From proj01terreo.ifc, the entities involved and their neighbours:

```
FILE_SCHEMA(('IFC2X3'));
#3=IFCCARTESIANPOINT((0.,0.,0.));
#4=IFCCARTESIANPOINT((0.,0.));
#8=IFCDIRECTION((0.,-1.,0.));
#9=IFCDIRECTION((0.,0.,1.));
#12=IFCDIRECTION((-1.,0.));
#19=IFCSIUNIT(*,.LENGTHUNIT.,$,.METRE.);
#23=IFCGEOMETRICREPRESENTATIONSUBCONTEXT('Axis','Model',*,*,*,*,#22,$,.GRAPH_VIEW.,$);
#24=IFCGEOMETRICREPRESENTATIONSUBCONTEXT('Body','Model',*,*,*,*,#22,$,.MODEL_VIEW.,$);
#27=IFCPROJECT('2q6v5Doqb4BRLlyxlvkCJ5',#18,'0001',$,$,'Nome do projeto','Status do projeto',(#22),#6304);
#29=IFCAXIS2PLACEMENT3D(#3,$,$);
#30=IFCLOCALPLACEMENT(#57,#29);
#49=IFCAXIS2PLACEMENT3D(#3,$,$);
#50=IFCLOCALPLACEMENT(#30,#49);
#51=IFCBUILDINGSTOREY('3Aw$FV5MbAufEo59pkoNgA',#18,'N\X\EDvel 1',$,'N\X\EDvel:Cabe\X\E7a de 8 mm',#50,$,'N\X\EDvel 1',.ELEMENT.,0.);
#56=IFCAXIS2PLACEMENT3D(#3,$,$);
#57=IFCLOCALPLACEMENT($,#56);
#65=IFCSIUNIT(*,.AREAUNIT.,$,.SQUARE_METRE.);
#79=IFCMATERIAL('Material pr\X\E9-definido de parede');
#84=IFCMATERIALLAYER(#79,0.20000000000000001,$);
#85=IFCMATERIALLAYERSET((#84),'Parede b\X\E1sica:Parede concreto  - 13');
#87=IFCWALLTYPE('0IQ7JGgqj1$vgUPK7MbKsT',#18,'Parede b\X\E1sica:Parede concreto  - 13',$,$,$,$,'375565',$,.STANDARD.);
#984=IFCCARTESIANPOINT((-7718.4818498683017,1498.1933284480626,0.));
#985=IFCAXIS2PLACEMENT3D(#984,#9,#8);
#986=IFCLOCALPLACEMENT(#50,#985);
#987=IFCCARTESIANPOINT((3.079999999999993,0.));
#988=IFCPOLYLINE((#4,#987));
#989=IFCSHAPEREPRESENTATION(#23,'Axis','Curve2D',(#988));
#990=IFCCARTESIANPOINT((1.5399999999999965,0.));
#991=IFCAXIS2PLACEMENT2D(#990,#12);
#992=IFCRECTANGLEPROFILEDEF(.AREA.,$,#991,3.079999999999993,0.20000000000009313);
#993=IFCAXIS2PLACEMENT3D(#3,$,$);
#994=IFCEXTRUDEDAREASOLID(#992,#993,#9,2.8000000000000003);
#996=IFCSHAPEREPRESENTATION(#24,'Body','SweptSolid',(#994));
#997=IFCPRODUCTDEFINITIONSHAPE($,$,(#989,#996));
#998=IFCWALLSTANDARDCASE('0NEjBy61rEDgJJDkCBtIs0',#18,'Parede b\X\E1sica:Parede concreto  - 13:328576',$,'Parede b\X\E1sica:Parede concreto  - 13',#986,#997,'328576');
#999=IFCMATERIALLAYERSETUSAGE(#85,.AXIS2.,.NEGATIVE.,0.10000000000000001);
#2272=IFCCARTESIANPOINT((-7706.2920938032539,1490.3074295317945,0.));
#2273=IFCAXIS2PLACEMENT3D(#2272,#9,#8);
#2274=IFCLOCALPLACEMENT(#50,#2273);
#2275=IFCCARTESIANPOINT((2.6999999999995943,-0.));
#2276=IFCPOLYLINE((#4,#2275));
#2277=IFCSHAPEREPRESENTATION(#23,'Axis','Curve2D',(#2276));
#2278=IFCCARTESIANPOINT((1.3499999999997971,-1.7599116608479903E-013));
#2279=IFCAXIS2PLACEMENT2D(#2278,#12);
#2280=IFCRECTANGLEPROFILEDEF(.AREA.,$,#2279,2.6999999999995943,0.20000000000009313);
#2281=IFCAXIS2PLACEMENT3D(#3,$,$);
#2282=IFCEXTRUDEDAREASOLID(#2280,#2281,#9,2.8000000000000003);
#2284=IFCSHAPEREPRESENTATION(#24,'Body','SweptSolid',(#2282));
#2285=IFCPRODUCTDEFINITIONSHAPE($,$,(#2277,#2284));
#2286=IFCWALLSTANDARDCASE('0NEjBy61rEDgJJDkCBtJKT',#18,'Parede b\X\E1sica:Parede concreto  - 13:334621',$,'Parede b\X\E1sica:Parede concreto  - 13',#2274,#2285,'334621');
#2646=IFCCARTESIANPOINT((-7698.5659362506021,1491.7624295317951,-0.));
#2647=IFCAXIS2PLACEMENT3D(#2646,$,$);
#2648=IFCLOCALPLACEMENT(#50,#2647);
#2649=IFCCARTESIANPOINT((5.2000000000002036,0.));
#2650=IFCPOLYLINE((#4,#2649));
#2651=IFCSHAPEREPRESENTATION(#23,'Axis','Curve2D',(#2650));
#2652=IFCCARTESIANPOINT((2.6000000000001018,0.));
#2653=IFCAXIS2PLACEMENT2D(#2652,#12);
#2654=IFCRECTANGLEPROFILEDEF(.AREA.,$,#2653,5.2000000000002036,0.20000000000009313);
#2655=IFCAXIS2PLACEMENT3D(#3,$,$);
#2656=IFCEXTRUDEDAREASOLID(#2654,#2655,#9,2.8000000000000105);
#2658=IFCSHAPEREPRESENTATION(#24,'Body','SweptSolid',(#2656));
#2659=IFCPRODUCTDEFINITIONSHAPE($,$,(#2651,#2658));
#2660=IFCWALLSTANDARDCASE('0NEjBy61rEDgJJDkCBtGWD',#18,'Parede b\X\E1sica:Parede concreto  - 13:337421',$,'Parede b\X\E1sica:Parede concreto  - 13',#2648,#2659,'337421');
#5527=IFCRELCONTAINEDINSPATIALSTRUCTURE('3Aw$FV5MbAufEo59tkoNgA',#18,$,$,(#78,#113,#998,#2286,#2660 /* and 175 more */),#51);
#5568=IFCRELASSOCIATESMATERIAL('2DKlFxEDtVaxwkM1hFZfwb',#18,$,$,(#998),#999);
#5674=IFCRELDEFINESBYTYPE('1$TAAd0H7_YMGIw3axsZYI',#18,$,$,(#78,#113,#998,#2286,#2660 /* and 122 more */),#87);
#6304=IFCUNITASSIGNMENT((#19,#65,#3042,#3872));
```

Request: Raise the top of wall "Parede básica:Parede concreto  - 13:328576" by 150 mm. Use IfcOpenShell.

```python
import ifcopenshell
import ifcopenshell.geom
import ifcopenshell.util.representation
import ifcopenshell.util.shape
import ifcopenshell.util.unit

model = ifcopenshell.open("proj01terreo.ifc")
unit_scale = ifcopenshell.util.unit.calculate_unit_scale(model)
settings = ifcopenshell.geom.settings()


def volume(element):
    """Net volume in cubic metres, openings subtracted."""
    shape = ifcopenshell.geom.create_shape(settings, element)
    return ifcopenshell.util.shape.get_volume(shape.geometry)


wall = model.by_guid("0NEjBy61rEDgJJDkCBtIs0")
before = volume(wall)

body = ifcopenshell.util.representation.get_representation(wall, "Model", "Body")
solid = body.Items[0]
old_height = solid.Depth
solid.Depth += 0.15 / unit_scale
after = volume(wall)

print(f"height {old_height:g} -> {solid.Depth:g}, volume {before:.3f} -> {after:.3f} m3")

model.write("proj01terreo_v2.ifc")
```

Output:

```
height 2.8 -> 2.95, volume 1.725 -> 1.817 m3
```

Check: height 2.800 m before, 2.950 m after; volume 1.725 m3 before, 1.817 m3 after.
